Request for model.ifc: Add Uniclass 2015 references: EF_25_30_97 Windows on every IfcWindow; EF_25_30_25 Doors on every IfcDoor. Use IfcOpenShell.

First a look at what the model holds.

```python
import ifcopenshell

model = ifcopenshell.open("model.ifc")
print(model.schema)
print("classifications:", [c.Name for c in model.by_type("IfcClassification")])
for ifc_class in ("IfcDoor", "IfcRoof", "IfcStair", "IfcWall", "IfcWindow"):
    print(ifc_class, len(model.by_type(ifc_class)))
```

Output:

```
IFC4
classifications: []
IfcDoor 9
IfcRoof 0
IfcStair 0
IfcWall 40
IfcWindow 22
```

```python
import ifcopenshell
import ifcopenshell.api.classification

model = ifcopenshell.open("model.ifc")

system = ifcopenshell.api.classification.add_classification(model, classification="Uniclass 2015")

codes = {
    "IfcWindow": ("EF_25_30_97", "Windows"),
    "IfcDoor": ("EF_25_30_25", "Doors"),
}
for ifc_class, (code, name) in codes.items():
    products = model.by_type(ifc_class)
    ifcopenshell.api.classification.add_reference(
        model, products=products, classification=system, identification=code, name=name
    )
    print(code, len(products))

model.write("model-out.ifc")
```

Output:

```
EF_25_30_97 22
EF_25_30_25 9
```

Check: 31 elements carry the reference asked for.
